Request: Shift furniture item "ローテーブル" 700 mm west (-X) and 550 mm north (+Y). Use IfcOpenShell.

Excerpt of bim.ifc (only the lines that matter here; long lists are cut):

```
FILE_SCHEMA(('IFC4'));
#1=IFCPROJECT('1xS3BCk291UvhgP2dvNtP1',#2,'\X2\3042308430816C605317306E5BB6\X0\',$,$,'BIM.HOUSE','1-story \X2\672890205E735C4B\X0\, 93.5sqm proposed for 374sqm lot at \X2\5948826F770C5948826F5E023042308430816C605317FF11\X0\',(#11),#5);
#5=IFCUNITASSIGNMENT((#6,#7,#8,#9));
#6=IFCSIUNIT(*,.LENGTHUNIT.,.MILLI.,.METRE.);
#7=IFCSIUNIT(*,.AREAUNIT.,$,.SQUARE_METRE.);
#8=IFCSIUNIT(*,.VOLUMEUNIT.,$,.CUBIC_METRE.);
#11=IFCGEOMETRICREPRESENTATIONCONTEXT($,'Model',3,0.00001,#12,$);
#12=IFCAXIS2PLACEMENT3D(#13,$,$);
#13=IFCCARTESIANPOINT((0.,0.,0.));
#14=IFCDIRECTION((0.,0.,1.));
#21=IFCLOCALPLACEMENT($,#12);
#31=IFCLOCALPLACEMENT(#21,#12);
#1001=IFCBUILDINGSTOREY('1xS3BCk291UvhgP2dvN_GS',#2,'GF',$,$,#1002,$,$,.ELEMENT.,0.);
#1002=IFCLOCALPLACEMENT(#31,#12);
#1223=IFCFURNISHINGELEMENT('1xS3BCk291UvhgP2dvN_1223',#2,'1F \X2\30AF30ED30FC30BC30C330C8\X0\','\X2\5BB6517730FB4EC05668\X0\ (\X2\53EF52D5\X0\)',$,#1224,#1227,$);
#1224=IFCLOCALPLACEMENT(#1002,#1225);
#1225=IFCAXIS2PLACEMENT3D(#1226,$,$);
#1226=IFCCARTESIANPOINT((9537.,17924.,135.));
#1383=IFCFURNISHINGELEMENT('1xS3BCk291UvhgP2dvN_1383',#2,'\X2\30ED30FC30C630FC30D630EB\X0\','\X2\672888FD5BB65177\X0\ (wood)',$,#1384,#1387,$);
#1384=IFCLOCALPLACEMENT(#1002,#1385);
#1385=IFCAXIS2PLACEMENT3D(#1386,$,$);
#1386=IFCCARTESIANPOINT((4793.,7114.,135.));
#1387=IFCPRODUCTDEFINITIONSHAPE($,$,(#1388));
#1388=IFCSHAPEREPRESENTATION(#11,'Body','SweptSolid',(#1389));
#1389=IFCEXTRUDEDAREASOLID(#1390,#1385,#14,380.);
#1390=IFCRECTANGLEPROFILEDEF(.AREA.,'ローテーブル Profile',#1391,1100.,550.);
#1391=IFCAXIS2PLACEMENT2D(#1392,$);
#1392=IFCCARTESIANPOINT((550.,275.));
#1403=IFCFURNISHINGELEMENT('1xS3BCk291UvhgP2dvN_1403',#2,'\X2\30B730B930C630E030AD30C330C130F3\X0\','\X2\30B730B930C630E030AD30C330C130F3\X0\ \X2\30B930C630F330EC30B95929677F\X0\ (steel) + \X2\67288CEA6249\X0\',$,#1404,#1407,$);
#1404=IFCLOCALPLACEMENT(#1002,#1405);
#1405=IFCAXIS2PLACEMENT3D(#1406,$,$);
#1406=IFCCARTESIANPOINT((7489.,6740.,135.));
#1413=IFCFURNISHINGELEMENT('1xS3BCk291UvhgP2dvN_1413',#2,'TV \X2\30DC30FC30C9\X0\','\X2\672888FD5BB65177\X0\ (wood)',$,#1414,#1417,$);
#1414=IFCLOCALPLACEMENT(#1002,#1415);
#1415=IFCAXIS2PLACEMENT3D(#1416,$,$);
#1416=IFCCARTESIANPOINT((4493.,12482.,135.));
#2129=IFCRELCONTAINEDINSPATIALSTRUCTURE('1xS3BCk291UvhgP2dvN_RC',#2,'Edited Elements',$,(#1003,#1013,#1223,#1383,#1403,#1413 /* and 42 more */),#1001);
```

```python
import ifcopenshell
import ifcopenshell.api.geometry
import ifcopenshell.util.placement
import ifcopenshell.util.unit

model = ifcopenshell.open("bim.ifc")
unit_scale = ifcopenshell.util.unit.calculate_unit_scale(model)

item = model.by_id(1383)
matrix = ifcopenshell.util.placement.get_local_placement(item.ObjectPlacement)
matrix[0, 3] -= 0.7 / unit_scale
matrix[1, 3] += 0.55 / unit_scale
ifcopenshell.api.geometry.edit_object_placement(model, product=item, matrix=matrix, is_si=False)

print(ifcopenshell.util.placement.get_local_placement(item.ObjectPlacement).round(3) + 0.0)

model.write("bim_rev.ifc")
```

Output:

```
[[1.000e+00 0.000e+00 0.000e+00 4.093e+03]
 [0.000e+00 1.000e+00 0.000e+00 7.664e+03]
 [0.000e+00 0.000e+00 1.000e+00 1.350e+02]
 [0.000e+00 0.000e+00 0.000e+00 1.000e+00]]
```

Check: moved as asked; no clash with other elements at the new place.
